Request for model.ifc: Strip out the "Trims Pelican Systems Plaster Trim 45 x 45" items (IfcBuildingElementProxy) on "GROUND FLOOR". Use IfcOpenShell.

First a look at what the model holds.

```python
import ifcopenshell
import ifcopenshell.util.element

model = ifcopenshell.open("model.ifc")
print(model.schema)
storey = next(s for s in model.by_type("IfcBuildingStorey") if s.Name == "GROUND FLOOR")
proxies = [e for e in ifcopenshell.util.element.get_decomposition(storey) if e.is_a("IfcBuildingElementProxy")]
seen = {}
for e in proxies:
    element_type = ifcopenshell.util.element.get_type(e)
    name = element_type.Name if element_type not in (None, e) else None
    seen[name] = seen.get(name, 0) + 1
for name, count in sorted(seen.items(), key=str):
    print(count, "x", name)
```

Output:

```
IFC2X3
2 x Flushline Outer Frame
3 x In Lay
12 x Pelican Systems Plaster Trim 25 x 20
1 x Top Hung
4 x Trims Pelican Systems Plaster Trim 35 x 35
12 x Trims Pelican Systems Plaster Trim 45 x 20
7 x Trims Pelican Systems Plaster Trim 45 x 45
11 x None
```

```python
import ifcopenshell
import ifcopenshell.api.root
import ifcopenshell.util.element

model = ifcopenshell.open("model.ifc")

storey = next(s for s in model.by_type("IfcBuildingStorey") if s.Name == "GROUND FLOOR")
proxies = [e for e in ifcopenshell.util.element.get_decomposition(storey) if e.is_a("IfcBuildingElementProxy")]
targets = [e for e in proxies if (t := ifcopenshell.util.element.get_type(e)) not in (None, e) and t.Name == "Trims Pelican Systems Plaster Trim 45 x 45"]

for e in targets:
    ifcopenshell.api.root.remove_product(model, product=e)
print(len(targets), "removed")

model.write("model-out.ifc")
```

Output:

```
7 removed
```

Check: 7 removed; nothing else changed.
